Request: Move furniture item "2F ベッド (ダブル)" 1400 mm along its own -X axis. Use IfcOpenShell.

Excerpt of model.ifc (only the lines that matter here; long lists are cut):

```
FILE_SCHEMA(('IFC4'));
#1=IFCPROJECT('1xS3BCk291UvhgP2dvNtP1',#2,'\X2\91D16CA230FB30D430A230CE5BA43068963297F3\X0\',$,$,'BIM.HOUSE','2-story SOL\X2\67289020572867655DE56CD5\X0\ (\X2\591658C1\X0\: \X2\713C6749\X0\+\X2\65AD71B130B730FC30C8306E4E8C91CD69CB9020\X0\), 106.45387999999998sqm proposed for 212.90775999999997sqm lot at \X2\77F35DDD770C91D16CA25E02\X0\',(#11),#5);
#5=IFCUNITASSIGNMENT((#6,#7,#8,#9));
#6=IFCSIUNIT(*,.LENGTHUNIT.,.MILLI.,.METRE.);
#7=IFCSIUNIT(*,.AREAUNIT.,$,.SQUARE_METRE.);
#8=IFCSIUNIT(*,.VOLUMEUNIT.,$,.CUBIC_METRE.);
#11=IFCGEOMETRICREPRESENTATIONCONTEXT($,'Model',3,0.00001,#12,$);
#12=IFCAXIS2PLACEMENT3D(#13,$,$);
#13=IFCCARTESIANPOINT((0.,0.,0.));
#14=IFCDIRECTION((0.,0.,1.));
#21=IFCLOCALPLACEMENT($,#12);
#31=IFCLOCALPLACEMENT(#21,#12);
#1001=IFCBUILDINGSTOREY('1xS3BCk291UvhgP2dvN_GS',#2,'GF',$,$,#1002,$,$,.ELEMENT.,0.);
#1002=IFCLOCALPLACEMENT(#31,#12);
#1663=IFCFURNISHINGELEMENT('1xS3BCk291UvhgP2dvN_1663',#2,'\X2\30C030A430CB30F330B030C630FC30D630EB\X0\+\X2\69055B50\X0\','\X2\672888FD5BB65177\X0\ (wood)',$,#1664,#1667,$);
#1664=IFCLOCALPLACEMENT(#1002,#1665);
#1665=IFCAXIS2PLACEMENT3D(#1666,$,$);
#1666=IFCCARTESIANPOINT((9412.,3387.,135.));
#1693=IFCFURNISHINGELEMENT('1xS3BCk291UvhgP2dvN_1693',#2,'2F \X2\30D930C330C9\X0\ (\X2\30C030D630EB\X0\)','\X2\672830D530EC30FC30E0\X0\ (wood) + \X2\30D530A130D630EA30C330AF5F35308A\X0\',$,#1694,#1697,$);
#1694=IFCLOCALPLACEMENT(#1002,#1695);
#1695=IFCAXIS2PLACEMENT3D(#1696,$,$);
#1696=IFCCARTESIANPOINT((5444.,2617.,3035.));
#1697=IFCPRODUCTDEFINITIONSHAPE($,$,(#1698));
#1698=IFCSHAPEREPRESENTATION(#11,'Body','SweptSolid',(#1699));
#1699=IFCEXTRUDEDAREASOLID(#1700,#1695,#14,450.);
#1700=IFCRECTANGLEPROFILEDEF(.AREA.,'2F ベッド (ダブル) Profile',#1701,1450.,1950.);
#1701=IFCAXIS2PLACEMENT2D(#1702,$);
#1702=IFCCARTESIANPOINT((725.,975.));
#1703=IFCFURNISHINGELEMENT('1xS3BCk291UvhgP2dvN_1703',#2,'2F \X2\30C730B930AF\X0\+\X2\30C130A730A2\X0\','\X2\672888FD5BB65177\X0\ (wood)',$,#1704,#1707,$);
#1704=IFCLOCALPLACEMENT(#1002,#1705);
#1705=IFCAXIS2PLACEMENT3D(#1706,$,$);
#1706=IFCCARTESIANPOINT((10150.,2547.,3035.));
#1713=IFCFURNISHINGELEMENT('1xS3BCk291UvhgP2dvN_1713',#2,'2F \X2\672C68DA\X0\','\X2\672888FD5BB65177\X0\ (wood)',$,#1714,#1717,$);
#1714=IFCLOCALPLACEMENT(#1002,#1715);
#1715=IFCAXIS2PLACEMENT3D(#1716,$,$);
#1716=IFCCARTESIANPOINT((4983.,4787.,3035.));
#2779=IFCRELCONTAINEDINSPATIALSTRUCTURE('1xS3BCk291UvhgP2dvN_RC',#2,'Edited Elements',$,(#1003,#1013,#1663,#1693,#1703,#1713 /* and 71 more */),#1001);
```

```python
import ifcopenshell
import ifcopenshell.api.geometry
import ifcopenshell.util.placement

model = ifcopenshell.open("model.ifc")

item = model.by_guid("1xS3BCk291UvhgP2dvN_1693")
matrix = ifcopenshell.util.placement.get_local_placement(item.ObjectPlacement)
matrix[:3, 3] -= matrix[:3, 0] * 1400.0
ifcopenshell.api.geometry.edit_object_placement(model, product=item, matrix=matrix, is_si=False)

print(ifcopenshell.util.placement.get_local_placement(item.ObjectPlacement).round(3) + 0.0)

model.write("model_edited.ifc")
```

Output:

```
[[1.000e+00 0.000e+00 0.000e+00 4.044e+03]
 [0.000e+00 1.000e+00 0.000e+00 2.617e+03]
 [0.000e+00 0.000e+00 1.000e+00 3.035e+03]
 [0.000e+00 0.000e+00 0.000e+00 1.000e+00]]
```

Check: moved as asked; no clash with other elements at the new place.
